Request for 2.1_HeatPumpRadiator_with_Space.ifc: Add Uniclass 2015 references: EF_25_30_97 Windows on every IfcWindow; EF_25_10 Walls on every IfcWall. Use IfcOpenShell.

First a look at what the model holds.

```python
import ifcopenshell

model = ifcopenshell.open("2.1_HeatPumpRadiator_with_Space.ifc")
print(model.schema)
print("classifications:", [c.Name for c in model.by_type("IfcClassification")])
for ifc_class in ("IfcDoor", "IfcRoof", "IfcStair", "IfcWall", "IfcWindow"):
    print(ifc_class, len(model.by_type(ifc_class)))
```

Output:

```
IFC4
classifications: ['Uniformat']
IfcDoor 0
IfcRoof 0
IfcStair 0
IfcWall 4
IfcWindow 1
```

```python
import ifcopenshell
import ifcopenshell.api.classification

model = ifcopenshell.open("2.1_HeatPumpRadiator_with_Space.ifc")

system = ifcopenshell.api.classification.add_classification(model, classification="Uniclass 2015")

codes = {
    "IfcWindow": ("EF_25_30_97", "Windows"),
    "IfcWall": ("EF_25_10", "Walls"),
}
for ifc_class, (code, name) in codes.items():
    products = model.by_type(ifc_class)
    ifcopenshell.api.classification.add_reference(
        model, products=products, classification=system, identification=code, name=name
    )
    print(code, len(products))

model.write("2.1_HeatPumpRadiator_with_Space_v2.ifc")
```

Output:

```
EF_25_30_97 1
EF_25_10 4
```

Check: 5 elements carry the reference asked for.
